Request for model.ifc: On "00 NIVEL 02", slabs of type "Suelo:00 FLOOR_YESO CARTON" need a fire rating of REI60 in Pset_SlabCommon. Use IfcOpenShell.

First a look at what the model holds.

```python
import ifcopenshell
import ifcopenshell.util.element

model = ifcopenshell.open("model.ifc")
print(model.schema)
storey = next(s for s in model.by_type("IfcBuildingStorey") if s.Name == "00 NIVEL 02")
slabs = [e for e in ifcopenshell.util.element.get_decomposition(storey) if e.is_a("IfcSlab")]
seen = {}
for e in slabs:
    element_type = ifcopenshell.util.element.get_type(e)
    key = (element_type.Name if element_type != e and element_type else None, ifcopenshell.util.element.get_pset(e, "Pset_SlabCommon", "FireRating"))
    seen[key] = seen.get(key, 0) + 1
for (name, value), count in sorted(seen.items(), key=str):
    print(count, "x", name, "|", value)
```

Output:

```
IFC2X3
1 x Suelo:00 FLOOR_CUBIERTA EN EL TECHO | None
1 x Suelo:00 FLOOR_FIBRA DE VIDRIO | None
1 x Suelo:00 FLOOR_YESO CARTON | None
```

```python
import ifcopenshell
import ifcopenshell.api.pset
import ifcopenshell.util.element

model = ifcopenshell.open("model.ifc")

storey = next(s for s in model.by_type("IfcBuildingStorey") if s.Name == "00 NIVEL 02")
slabs = [e for e in ifcopenshell.util.element.get_decomposition(storey) if e.is_a("IfcSlab")]

count = 0
for e in slabs:
    element_type = ifcopenshell.util.element.get_type(e)
    if element_type in (None, e) or element_type.Name != "Suelo:00 FLOOR_YESO CARTON":
        continue
    # add_pset returns the element's existing set when there is one.
    pset = ifcopenshell.api.pset.add_pset(model, product=e, name="Pset_SlabCommon")
    ifcopenshell.api.pset.edit_pset(model, pset=pset, properties={"FireRating": "REI60"})
    count += 1

print(count, "slabs updated")

model.write("model_v2.ifc")
```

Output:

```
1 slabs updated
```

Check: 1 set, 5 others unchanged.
